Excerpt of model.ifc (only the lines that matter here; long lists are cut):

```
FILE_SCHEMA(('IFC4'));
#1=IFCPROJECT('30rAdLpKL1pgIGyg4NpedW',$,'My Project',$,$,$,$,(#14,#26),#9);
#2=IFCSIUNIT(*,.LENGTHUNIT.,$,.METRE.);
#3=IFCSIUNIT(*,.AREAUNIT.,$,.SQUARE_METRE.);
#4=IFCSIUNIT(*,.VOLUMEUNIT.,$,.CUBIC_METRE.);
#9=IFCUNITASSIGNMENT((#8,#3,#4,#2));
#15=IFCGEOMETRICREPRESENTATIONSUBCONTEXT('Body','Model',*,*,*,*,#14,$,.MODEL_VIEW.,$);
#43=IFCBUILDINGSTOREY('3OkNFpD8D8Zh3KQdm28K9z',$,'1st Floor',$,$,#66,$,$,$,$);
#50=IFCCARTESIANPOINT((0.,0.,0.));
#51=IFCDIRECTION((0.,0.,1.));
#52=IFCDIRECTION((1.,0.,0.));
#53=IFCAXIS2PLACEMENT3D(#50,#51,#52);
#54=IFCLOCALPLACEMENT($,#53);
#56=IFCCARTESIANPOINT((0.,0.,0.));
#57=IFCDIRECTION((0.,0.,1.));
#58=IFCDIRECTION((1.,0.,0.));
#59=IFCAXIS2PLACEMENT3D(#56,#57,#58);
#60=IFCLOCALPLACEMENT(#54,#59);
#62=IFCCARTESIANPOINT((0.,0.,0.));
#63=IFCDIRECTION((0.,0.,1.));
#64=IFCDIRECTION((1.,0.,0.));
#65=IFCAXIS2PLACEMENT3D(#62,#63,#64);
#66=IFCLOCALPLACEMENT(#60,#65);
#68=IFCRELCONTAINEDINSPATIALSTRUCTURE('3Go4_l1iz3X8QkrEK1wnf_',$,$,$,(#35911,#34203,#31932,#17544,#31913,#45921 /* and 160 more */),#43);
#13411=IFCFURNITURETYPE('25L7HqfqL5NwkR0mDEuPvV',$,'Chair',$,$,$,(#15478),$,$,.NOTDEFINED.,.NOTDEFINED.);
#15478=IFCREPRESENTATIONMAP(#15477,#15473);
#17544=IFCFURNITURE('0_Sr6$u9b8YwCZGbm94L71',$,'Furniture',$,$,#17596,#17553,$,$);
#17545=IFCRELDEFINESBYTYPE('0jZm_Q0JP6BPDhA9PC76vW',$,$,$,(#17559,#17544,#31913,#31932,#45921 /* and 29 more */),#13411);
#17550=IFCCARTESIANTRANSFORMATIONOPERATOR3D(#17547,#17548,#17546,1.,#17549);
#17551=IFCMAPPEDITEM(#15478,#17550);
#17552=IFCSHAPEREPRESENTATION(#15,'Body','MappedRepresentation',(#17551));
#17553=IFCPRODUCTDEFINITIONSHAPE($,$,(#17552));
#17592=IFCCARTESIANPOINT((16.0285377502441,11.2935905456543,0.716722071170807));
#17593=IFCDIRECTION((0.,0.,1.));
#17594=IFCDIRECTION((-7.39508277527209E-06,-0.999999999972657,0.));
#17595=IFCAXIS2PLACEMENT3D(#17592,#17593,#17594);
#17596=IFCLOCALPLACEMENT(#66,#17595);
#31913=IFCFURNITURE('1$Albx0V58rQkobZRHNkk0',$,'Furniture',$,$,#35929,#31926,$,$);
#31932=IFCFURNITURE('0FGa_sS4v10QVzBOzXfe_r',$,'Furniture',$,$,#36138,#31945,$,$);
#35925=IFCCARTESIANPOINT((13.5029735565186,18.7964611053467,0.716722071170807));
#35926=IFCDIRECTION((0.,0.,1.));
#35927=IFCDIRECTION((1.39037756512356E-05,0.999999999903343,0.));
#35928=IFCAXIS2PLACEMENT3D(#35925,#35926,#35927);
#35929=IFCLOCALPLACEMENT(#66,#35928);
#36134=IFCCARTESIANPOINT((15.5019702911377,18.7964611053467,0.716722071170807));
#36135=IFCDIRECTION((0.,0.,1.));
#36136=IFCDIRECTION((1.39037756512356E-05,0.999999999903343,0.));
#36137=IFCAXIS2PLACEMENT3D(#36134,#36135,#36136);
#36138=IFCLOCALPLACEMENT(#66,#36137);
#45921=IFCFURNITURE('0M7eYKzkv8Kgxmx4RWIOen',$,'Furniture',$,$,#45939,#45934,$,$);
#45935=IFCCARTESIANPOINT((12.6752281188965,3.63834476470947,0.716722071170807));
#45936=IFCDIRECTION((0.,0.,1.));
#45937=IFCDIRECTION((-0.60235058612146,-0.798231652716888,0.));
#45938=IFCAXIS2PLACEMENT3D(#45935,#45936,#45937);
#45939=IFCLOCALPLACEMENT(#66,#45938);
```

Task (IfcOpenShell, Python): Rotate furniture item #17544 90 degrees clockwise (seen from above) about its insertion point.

```python
import ifcopenshell
import ifcopenshell.api.geometry
import ifcopenshell.util.placement

model = ifcopenshell.open("model.ifc")

item = model.by_guid("0_Sr6$u9b8YwCZGbm94L71")
matrix = ifcopenshell.util.placement.get_local_placement(item.ObjectPlacement)
matrix = matrix @ ifcopenshell.util.placement.rotation(-90, "Z")
ifcopenshell.api.geometry.edit_object_placement(model, product=item, matrix=matrix, is_si=False)

print(ifcopenshell.util.placement.get_local_placement(item.ObjectPlacement).round(3) + 0.0)

model.write("model_rev.ifc")
```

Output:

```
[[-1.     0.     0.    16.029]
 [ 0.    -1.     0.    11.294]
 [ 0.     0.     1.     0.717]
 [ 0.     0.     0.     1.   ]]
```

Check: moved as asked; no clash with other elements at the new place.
